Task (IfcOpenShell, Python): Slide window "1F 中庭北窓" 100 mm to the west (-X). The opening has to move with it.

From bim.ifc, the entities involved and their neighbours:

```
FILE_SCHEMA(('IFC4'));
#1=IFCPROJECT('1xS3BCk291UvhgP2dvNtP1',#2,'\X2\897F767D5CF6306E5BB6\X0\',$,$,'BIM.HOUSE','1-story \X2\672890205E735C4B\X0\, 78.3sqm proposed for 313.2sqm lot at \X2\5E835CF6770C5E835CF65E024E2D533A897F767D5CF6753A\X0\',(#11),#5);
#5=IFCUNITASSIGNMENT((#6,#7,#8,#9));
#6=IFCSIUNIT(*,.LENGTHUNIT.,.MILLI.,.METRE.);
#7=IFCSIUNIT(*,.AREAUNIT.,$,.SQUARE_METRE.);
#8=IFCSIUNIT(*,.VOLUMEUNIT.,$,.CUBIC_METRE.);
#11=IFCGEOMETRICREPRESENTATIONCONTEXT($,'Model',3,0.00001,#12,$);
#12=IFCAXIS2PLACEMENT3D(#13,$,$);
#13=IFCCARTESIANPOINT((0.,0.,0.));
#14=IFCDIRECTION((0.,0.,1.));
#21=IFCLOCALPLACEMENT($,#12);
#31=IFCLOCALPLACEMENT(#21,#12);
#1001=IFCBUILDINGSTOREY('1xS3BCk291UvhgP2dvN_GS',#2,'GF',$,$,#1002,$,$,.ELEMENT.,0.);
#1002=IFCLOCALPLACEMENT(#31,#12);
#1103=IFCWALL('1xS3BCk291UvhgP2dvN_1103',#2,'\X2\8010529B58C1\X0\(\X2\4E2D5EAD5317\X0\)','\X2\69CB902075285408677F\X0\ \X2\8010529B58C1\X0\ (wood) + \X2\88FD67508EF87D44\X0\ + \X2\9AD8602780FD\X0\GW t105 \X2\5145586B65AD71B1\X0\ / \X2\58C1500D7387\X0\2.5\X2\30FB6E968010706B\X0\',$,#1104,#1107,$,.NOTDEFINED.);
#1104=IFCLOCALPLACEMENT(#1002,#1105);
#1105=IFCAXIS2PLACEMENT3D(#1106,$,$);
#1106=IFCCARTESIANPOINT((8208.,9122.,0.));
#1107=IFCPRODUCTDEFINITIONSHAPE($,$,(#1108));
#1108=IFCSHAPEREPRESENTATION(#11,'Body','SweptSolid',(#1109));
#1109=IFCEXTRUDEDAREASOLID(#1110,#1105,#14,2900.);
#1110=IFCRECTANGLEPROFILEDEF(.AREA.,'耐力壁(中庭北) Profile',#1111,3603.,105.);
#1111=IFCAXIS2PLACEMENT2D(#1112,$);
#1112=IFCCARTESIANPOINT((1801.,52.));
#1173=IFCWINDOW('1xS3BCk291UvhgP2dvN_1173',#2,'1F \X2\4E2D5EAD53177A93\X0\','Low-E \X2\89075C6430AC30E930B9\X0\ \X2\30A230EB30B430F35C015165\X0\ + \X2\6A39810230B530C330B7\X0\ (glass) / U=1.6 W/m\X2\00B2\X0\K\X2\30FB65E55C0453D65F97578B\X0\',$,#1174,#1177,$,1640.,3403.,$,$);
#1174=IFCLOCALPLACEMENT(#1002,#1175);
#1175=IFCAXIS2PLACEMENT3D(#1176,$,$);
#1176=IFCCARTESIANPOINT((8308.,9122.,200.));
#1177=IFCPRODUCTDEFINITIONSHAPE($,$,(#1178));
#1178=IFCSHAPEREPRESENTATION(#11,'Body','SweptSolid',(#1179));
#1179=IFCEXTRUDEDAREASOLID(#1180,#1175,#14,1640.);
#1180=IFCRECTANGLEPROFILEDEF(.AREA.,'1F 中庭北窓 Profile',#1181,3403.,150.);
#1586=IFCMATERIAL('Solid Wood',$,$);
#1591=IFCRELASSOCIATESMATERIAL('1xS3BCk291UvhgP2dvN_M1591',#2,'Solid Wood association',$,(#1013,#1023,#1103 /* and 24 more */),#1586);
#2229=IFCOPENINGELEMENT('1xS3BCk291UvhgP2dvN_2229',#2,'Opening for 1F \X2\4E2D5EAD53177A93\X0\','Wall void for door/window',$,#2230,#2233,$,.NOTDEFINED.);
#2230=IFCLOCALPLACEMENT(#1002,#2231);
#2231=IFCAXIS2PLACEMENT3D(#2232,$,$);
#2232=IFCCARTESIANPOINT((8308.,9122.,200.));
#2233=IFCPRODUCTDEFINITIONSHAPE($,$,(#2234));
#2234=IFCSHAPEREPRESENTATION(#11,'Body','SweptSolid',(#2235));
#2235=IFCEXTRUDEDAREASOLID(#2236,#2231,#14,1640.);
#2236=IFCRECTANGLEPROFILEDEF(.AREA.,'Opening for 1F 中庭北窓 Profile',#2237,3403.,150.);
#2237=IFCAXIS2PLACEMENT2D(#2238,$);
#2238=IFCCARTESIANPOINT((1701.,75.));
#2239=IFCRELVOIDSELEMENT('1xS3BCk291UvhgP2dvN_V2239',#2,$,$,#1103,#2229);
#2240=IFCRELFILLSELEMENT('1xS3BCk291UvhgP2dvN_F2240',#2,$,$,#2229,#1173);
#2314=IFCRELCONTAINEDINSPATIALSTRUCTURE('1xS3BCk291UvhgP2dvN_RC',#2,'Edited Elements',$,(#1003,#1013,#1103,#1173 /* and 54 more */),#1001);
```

```python
import ifcopenshell
import ifcopenshell.api.geometry
import ifcopenshell.util.placement

model = ifcopenshell.open("bim.ifc")

window = model.by_guid("1xS3BCk291UvhgP2dvN_1173")
opening = window.FillsVoids[0].RelatingOpeningElement
wall = opening.VoidsElements[0].RelatingBuildingElement

wall_matrix = ifcopenshell.util.placement.get_local_placement(wall.ObjectPlacement)
shift = wall_matrix[:3, 0] * -100.0
before = ifcopenshell.util.placement.get_local_placement(window.ObjectPlacement)[:3, 3].copy()

# The window is not placed relative to its opening, so move both.
for product in (opening, window):
    matrix = ifcopenshell.util.placement.get_local_placement(product.ObjectPlacement)
    matrix[:3, 3] += shift
    ifcopenshell.api.geometry.edit_object_placement(model, product=product, matrix=matrix, is_si=False)

after = ifcopenshell.util.placement.get_local_placement(window.ObjectPlacement)[:3, 3]
print("window moved by", (after - before).round(3) + 0.0)

model.write("bim_rev.ifc")
```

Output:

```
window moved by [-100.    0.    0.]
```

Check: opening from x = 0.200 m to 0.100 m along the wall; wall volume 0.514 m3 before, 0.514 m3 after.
